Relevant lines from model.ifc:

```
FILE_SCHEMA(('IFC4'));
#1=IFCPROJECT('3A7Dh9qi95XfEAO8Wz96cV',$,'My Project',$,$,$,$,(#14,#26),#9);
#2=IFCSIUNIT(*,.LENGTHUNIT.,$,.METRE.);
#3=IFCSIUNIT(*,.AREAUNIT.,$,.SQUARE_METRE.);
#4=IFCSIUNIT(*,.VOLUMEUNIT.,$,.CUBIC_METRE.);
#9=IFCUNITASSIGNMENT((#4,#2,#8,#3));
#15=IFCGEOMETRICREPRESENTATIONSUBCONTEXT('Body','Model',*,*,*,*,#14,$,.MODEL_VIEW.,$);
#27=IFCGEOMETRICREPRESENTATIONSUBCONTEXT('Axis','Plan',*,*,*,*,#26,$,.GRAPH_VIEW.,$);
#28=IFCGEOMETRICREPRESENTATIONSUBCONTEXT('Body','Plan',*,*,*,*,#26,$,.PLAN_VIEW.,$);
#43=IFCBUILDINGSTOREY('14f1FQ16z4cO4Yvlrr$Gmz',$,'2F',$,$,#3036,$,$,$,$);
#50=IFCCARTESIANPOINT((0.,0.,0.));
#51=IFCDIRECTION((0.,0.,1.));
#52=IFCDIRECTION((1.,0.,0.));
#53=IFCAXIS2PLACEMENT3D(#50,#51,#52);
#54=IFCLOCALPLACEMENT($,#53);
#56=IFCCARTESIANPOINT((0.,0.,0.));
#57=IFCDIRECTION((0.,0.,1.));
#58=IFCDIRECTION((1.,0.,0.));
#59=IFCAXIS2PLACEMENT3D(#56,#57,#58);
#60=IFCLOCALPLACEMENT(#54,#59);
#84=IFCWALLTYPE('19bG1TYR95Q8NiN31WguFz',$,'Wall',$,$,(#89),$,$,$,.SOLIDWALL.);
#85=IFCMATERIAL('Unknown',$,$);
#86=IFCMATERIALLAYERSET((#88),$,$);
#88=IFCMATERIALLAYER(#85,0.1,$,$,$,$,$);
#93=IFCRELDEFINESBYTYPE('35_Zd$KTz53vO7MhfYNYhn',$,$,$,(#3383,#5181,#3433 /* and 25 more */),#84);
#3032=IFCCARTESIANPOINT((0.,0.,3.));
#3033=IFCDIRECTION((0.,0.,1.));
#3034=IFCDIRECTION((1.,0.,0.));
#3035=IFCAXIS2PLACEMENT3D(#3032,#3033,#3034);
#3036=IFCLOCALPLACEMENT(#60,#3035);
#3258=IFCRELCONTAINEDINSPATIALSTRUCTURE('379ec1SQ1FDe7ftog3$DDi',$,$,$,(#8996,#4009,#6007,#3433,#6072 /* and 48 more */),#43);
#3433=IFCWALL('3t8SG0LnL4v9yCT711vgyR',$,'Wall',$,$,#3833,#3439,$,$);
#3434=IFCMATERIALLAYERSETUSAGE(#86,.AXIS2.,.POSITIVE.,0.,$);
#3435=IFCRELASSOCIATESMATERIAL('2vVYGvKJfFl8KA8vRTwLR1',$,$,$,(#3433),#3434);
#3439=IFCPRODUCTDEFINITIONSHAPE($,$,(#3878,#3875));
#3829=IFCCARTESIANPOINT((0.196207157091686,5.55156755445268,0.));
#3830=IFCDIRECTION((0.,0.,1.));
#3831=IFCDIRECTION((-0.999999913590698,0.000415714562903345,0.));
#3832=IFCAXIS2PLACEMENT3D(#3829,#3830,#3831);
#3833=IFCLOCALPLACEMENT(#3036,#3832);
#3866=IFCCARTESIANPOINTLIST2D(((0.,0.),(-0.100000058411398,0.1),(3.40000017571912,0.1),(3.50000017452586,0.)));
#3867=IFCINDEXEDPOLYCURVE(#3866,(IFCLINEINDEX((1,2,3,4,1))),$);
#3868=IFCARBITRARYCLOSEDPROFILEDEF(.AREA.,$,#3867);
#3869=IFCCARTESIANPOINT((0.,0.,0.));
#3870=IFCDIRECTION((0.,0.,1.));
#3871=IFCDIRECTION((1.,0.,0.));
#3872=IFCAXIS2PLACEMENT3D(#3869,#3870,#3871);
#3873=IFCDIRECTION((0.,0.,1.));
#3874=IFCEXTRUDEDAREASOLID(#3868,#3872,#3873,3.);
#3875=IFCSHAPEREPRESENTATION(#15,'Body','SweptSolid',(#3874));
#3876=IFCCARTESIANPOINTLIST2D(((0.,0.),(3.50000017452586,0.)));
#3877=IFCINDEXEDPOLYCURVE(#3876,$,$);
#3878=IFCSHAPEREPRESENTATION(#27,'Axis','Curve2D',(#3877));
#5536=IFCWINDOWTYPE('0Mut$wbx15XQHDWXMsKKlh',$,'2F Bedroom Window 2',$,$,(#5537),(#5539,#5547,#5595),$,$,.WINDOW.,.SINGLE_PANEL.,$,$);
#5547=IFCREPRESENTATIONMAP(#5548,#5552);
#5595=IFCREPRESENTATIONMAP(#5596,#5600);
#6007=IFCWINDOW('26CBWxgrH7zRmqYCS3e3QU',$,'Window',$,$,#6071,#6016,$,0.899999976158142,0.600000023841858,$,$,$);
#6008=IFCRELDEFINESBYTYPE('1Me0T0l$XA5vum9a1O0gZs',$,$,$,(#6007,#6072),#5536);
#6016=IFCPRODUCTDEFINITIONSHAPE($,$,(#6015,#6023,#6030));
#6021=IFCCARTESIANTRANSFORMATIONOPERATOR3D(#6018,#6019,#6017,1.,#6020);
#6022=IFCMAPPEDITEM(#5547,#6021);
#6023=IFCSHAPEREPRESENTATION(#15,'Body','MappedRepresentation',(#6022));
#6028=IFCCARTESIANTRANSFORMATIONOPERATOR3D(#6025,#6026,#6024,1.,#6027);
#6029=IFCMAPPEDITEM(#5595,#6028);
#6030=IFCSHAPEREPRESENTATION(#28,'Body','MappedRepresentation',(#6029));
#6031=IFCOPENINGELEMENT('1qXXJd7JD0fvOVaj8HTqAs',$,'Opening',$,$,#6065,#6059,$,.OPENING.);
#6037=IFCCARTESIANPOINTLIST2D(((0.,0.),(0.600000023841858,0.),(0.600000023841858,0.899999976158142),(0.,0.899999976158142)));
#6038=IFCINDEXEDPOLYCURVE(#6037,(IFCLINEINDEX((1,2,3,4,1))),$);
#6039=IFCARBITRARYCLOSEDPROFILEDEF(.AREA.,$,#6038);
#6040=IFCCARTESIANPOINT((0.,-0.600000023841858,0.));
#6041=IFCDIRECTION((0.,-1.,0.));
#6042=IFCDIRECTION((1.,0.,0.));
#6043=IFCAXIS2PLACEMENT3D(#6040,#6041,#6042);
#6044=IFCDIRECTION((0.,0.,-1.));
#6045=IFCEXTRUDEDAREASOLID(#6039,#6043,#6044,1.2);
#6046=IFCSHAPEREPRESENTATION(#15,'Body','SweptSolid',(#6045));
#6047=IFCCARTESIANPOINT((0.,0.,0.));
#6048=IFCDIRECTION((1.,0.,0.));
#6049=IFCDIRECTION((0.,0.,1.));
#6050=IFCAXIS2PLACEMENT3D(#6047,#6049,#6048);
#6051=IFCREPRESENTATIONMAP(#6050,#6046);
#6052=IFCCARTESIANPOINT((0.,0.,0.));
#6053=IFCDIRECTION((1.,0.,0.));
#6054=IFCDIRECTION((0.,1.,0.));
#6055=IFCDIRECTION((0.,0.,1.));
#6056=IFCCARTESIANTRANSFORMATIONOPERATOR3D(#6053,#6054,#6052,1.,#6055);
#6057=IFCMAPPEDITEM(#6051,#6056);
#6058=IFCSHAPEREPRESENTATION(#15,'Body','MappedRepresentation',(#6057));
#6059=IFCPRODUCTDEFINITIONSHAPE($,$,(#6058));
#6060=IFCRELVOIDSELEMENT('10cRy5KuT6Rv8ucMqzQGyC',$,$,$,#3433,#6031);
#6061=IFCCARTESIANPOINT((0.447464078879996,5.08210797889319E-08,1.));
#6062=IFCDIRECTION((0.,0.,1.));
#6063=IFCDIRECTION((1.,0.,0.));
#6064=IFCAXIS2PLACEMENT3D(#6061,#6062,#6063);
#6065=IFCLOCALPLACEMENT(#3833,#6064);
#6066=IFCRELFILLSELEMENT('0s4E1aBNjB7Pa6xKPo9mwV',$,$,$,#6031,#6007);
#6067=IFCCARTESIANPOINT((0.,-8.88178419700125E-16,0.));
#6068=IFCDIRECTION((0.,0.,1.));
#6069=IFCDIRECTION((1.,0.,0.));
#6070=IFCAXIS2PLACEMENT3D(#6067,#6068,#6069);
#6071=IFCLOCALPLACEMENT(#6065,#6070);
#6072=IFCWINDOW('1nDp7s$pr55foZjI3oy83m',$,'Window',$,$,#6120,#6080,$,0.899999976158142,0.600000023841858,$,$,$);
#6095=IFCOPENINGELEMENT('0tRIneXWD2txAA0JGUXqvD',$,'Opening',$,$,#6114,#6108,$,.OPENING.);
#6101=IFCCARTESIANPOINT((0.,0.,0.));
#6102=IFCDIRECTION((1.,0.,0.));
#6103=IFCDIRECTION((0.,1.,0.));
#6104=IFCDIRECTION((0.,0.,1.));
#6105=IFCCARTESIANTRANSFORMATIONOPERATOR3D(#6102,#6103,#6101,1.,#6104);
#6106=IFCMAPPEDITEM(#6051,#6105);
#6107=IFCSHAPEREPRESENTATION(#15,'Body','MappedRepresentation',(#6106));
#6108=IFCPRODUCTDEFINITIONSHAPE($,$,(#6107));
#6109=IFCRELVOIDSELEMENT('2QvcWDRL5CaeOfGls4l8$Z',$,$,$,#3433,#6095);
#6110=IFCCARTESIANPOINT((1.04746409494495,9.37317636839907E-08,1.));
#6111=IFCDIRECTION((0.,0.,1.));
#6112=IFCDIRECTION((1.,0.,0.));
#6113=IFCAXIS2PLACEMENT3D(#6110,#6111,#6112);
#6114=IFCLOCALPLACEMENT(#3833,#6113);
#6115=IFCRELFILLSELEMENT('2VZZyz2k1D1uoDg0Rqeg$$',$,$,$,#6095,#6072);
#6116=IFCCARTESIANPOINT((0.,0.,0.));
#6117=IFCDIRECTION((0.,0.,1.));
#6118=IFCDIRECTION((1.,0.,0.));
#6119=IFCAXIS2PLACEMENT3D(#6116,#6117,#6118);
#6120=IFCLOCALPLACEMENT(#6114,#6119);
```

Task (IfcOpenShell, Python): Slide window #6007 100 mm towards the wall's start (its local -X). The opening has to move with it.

```python
import ifcopenshell
import ifcopenshell.api.geometry
import ifcopenshell.util.placement
import ifcopenshell.util.unit

model = ifcopenshell.open("model.ifc")
unit_scale = ifcopenshell.util.unit.calculate_unit_scale(model)

window = model.by_guid("26CBWxgrH7zRmqYCS3e3QU")
opening = window.FillsVoids[0].RelatingOpeningElement
wall = opening.VoidsElements[0].RelatingBuildingElement

wall_matrix = ifcopenshell.util.placement.get_local_placement(wall.ObjectPlacement)
shift = wall_matrix[:3, 0] * -0.1 / unit_scale
before = ifcopenshell.util.placement.get_local_placement(window.ObjectPlacement)[:3, 3].copy()

# The window is placed relative to its opening, so it follows when the opening moves.
matrix = ifcopenshell.util.placement.get_local_placement(opening.ObjectPlacement)
matrix[:3, 3] += shift
ifcopenshell.api.geometry.edit_object_placement(
    model, product=opening, matrix=matrix, is_si=False, should_transform_children=True
)

after = ifcopenshell.util.placement.get_local_placement(window.ObjectPlacement)[:3, 3]
print("window moved by", (after - before).round(3) + 0.0)

model.write("model_edited.ifc")
```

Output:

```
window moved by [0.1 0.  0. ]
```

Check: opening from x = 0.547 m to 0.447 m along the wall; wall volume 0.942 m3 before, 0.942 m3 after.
